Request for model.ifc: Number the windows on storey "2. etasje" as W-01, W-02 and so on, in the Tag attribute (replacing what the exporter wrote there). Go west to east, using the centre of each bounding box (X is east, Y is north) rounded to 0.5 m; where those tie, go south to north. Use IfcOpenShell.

First a look at what the model holds.

```python
import ifcopenshell
import ifcopenshell.util.element
import ifcopenshell.util.placement

model = ifcopenshell.open("model.ifc")
print(model.schema)
storey = next(s for s in model.by_type("IfcBuildingStorey") if s.Name == "2. etasje")
windows = [e for e in ifcopenshell.util.element.get_decomposition(storey) if e.is_a("IfcWindow")]
for e in sorted(windows, key=lambda e: e.id()):
    origin = ifcopenshell.util.placement.get_local_placement(e.ObjectPlacement)[:3, 3]
    print(e.id(), e.Tag, e.Name, origin.round(2) + 0.0, sep=" | ")
```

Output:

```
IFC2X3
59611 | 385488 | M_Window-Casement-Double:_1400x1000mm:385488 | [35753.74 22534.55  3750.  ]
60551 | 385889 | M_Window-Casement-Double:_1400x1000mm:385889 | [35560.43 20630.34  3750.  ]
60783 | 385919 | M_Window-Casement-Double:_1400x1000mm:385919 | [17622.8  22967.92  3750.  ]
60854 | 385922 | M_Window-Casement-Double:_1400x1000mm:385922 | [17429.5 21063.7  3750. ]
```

```python
import ifcopenshell
import ifcopenshell.geom
import ifcopenshell.util.element
import ifcopenshell.util.shape

model = ifcopenshell.open("model.ifc")
settings = ifcopenshell.geom.settings()
settings.set("use-world-coords", True)


def centre(element):
    shape = ifcopenshell.geom.create_shape(settings, element)
    return ifcopenshell.util.shape.get_bbox_centroid(shape.geometry)


storey = next(s for s in model.by_type("IfcBuildingStorey") if s.Name == "2. etasje")
windows = [e for e in ifcopenshell.util.element.get_decomposition(storey) if e.is_a("IfcWindow")]

# Insertion points can sit at a corner or the storey origin, so sort by the geometry (in metres).
centres = {e: centre(e) for e in windows}
windows.sort(key=lambda e: (round(centres[e][0] / 0.5), centres[e][1]))

for i, e in enumerate(windows, start=1):
    number = f"W-{i:02d}"
    e.Tag = number
    print(e.id(), number)

model.write("model-out.ifc")
```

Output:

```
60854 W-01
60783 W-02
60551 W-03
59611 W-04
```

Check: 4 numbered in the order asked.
